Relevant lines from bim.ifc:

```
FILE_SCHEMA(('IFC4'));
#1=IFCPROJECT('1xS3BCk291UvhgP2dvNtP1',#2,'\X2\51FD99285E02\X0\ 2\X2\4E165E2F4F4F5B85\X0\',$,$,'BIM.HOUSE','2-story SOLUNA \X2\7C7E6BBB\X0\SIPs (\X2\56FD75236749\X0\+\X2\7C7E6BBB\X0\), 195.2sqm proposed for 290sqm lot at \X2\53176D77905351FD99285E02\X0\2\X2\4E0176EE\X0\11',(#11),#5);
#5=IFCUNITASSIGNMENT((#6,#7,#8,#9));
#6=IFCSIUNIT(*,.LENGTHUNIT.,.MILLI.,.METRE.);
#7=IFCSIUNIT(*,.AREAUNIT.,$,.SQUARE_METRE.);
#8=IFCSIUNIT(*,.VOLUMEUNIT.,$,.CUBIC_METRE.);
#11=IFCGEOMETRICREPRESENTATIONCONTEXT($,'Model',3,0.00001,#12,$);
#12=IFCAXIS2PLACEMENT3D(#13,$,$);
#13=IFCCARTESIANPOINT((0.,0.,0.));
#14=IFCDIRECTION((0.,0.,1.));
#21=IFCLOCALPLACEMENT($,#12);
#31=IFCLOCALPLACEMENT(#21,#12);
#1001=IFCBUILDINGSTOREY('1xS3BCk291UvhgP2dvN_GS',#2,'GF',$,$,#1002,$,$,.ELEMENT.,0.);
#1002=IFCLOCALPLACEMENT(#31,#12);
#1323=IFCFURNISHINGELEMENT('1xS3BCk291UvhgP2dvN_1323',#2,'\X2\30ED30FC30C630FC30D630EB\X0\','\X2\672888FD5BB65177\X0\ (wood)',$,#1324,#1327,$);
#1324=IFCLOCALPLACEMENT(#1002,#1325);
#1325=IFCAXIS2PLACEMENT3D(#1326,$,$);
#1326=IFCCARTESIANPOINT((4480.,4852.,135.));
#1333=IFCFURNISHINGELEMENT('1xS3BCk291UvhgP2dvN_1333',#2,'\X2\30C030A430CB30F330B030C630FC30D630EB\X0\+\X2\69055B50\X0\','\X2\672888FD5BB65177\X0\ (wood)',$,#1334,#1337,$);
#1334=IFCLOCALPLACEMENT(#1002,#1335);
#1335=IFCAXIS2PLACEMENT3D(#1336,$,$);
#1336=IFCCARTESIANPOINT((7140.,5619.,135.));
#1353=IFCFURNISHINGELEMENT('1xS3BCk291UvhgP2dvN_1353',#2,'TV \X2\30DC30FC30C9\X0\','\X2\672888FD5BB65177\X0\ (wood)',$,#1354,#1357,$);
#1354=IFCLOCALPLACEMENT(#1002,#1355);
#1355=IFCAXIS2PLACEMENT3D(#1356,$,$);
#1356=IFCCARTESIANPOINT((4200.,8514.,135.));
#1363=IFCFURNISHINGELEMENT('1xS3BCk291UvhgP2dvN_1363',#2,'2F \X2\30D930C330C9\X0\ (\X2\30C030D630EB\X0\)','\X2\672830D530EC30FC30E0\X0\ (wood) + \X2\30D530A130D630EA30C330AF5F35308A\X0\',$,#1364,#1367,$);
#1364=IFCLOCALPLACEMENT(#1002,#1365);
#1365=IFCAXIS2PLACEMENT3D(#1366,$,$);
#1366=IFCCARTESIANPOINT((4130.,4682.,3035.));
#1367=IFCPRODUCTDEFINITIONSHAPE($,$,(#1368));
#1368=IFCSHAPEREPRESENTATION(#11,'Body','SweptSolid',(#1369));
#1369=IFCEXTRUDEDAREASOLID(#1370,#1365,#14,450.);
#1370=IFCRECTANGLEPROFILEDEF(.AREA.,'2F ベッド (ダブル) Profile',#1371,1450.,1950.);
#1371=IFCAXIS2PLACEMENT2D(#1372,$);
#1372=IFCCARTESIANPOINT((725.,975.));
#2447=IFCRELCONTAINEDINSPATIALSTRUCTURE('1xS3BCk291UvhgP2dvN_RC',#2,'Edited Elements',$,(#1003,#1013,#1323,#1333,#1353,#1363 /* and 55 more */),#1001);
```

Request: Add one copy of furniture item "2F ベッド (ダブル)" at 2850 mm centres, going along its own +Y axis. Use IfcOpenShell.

```python
import ifcopenshell
import ifcopenshell.api.geometry
import ifcopenshell.api.root
import ifcopenshell.util.element
import ifcopenshell.util.placement
import ifcopenshell.util.unit

model = ifcopenshell.open("bim.ifc")
unit_scale = ifcopenshell.util.unit.calculate_unit_scale(model)


def reuse_history(source, copy):
    """copy_class also copies each property set's owner history, people and application; keep the originals."""
    for rel in copy.IsDefinedBy:
        if rel.is_a("IfcRelDefinesByProperties") and (history := rel.RelatingPropertyDefinition.OwnerHistory):
            rel.RelatingPropertyDefinition.OwnerHistory = source.OwnerHistory
            ifcopenshell.util.element.remove_deep2(model, history)


source = model.by_id(1363)
base = ifcopenshell.util.placement.get_local_placement(source.ObjectPlacement)
step = base[:3, 1] * 2.85 / unit_scale

for i in range(1, 2):
    copy = ifcopenshell.api.root.copy_class(model, product=source)
    copy.Representation = ifcopenshell.util.element.copy_deep(
        model, source.Representation, exclude=["IfcGeometricRepresentationContext", "IfcRepresentationMap"]
    )
    reuse_history(source, copy)
    matrix = base.copy()
    matrix[:3, 3] += i * step
    print("added at", matrix[:3, 3].round(3) + 0.0)
    ifcopenshell.api.geometry.edit_object_placement(model, product=copy, matrix=matrix, is_si=False)

model.write("bim_edited.ifc")
```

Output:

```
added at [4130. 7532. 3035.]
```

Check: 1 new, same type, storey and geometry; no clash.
